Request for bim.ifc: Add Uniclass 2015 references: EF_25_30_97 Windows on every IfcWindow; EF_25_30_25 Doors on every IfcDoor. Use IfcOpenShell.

First a look at what the model holds.

```python
import ifcopenshell

model = ifcopenshell.open("bim.ifc")
print(model.schema)
print("classifications:", [c.Name for c in model.by_type("IfcClassification")])
for ifc_class in ("IfcDoor", "IfcRoof", "IfcStair", "IfcWall", "IfcWindow"):
    print(ifc_class, len(model.by_type(ifc_class)))
```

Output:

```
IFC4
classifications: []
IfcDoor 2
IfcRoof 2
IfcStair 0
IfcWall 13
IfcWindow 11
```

```python
import ifcopenshell
import ifcopenshell.api.classification

model = ifcopenshell.open("bim.ifc")

system = ifcopenshell.api.classification.add_classification(model, classification="Uniclass 2015")

codes = {
    "IfcWindow": ("EF_25_30_97", "Windows"),
    "IfcDoor": ("EF_25_30_25", "Doors"),
}
for ifc_class, (code, name) in codes.items():
    products = model.by_type(ifc_class)
    ifcopenshell.api.classification.add_reference(
        model, products=products, classification=system, identification=code, name=name
    )
    print(code, len(products))

model.write("bim-out.ifc")
```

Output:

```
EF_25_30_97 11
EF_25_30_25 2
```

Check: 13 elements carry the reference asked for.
